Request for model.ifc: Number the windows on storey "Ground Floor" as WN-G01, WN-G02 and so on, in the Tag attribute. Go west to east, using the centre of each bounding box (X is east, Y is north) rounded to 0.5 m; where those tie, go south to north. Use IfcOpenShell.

First a look at what the model holds.

```python
import ifcopenshell
import ifcopenshell.util.element
import ifcopenshell.util.placement

model = ifcopenshell.open("model.ifc")
print(model.schema)
storey = next(s for s in model.by_type("IfcBuildingStorey") if s.Name == "Ground Floor")
windows = [e for e in ifcopenshell.util.element.get_decomposition(storey) if e.is_a("IfcWindow")]
for e in sorted(windows, key=lambda e: e.id()):
    origin = ifcopenshell.util.placement.get_local_placement(e.ObjectPlacement)[:3, 3]
    print(e.id(), e.Tag, e.Name, origin.round(2) + 0.0, sep=" | ")
```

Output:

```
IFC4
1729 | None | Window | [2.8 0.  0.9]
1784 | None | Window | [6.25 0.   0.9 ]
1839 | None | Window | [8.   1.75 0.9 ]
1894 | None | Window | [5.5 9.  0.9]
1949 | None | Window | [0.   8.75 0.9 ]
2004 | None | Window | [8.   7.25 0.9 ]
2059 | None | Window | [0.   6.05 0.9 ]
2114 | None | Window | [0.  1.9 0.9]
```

```python
import ifcopenshell
import ifcopenshell.geom
import ifcopenshell.util.element
import ifcopenshell.util.shape

model = ifcopenshell.open("model.ifc")
settings = ifcopenshell.geom.settings()
settings.set("use-world-coords", True)


def centre(element):
    shape = ifcopenshell.geom.create_shape(settings, element)
    return ifcopenshell.util.shape.get_bbox_centroid(shape.geometry)


storey = next(s for s in model.by_type("IfcBuildingStorey") if s.Name == "Ground Floor")
windows = [e for e in ifcopenshell.util.element.get_decomposition(storey) if e.is_a("IfcWindow")]

# Insertion points can sit at a corner or the storey origin, so sort by the geometry (in metres).
centres = {e: centre(e) for e in windows}
windows.sort(key=lambda e: (round(centres[e][0] / 0.5), centres[e][1]))

for i, e in enumerate(windows, start=1):
    number = f"WN-G{i:02d}"
    e.Tag = number
    print(e.id(), number)

model.write("model_rev.ifc")
```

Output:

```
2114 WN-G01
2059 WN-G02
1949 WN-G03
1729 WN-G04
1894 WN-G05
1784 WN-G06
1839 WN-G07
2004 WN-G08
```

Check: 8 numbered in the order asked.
